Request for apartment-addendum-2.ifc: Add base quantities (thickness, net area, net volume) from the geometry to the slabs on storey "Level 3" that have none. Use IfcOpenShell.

First a look at what the model holds.

```python
import ifcopenshell
import ifcopenshell.util.element
import ifcopenshell.util.unit

model = ifcopenshell.open("apartment-addendum-2.ifc")
print(model.schema)
for unit_type in ("LENGTHUNIT", "AREAUNIT", "VOLUMEUNIT"):
    print(unit_type, ifcopenshell.util.unit.calculate_unit_scale(model, unit_type))
storey = next(s for s in model.by_type("IfcBuildingStorey") if s.Name == "Level 3")
slabs = [e for e in ifcopenshell.util.element.get_decomposition(storey) if e.is_a("IfcSlab")]
for e in sorted(slabs, key=lambda e: e.id()):
    print(e.id(), e.is_a(), e.Name, list(ifcopenshell.util.element.get_psets(e, qtos_only=True)), sep=" | ")
```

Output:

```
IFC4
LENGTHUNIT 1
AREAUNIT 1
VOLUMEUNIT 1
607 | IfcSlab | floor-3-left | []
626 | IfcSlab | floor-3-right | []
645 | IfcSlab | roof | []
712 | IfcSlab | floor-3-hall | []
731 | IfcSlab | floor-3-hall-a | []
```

```python
import ifcopenshell
import ifcopenshell.api.pset
import ifcopenshell.geom
import ifcopenshell.util.element
import ifcopenshell.util.shape
import ifcopenshell.util.unit

model = ifcopenshell.open("apartment-addendum-2.ifc")
unit_scale = ifcopenshell.util.unit.calculate_unit_scale(model)
area_scale = ifcopenshell.util.unit.calculate_unit_scale(model, "AREAUNIT")
volume_scale = ifcopenshell.util.unit.calculate_unit_scale(model, "VOLUMEUNIT")
settings = ifcopenshell.geom.settings()

storey = next(s for s in model.by_type("IfcBuildingStorey") if s.Name == "Level 3")
slabs = [e for e in ifcopenshell.util.element.get_decomposition(storey) if e.is_a("IfcSlab")]

for e in sorted(slabs, key=lambda e: e.id()):
    if ifcopenshell.util.element.get_psets(e, qtos_only=True, should_inherit=False):
        continue
    # Geometry comes back in metres, in the element's own axes.
    shape = ifcopenshell.geom.create_shape(settings, e)
    values = {
        "Width": ifcopenshell.util.shape.get_z(shape.geometry) / unit_scale,
        "NetArea": ifcopenshell.util.shape.get_footprint_area(shape.geometry) / area_scale,
        "NetVolume": ifcopenshell.util.shape.get_volume(shape.geometry) / volume_scale,
    }
    qto = ifcopenshell.api.pset.add_qto(model, product=e, name="Qto_SlabBaseQuantities")
    ifcopenshell.api.pset.edit_qto(model, qto=qto, properties=values)
    print(e.id(), {k: round(v, 3) for k, v in values.items()})

model.write("apartment-addendum-2_edited.ifc")
```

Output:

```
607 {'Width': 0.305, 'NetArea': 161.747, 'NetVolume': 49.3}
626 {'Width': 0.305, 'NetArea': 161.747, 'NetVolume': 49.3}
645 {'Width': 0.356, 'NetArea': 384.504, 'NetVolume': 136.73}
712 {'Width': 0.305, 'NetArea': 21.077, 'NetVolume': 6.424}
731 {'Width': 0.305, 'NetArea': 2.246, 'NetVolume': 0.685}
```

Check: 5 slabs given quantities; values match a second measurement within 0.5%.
